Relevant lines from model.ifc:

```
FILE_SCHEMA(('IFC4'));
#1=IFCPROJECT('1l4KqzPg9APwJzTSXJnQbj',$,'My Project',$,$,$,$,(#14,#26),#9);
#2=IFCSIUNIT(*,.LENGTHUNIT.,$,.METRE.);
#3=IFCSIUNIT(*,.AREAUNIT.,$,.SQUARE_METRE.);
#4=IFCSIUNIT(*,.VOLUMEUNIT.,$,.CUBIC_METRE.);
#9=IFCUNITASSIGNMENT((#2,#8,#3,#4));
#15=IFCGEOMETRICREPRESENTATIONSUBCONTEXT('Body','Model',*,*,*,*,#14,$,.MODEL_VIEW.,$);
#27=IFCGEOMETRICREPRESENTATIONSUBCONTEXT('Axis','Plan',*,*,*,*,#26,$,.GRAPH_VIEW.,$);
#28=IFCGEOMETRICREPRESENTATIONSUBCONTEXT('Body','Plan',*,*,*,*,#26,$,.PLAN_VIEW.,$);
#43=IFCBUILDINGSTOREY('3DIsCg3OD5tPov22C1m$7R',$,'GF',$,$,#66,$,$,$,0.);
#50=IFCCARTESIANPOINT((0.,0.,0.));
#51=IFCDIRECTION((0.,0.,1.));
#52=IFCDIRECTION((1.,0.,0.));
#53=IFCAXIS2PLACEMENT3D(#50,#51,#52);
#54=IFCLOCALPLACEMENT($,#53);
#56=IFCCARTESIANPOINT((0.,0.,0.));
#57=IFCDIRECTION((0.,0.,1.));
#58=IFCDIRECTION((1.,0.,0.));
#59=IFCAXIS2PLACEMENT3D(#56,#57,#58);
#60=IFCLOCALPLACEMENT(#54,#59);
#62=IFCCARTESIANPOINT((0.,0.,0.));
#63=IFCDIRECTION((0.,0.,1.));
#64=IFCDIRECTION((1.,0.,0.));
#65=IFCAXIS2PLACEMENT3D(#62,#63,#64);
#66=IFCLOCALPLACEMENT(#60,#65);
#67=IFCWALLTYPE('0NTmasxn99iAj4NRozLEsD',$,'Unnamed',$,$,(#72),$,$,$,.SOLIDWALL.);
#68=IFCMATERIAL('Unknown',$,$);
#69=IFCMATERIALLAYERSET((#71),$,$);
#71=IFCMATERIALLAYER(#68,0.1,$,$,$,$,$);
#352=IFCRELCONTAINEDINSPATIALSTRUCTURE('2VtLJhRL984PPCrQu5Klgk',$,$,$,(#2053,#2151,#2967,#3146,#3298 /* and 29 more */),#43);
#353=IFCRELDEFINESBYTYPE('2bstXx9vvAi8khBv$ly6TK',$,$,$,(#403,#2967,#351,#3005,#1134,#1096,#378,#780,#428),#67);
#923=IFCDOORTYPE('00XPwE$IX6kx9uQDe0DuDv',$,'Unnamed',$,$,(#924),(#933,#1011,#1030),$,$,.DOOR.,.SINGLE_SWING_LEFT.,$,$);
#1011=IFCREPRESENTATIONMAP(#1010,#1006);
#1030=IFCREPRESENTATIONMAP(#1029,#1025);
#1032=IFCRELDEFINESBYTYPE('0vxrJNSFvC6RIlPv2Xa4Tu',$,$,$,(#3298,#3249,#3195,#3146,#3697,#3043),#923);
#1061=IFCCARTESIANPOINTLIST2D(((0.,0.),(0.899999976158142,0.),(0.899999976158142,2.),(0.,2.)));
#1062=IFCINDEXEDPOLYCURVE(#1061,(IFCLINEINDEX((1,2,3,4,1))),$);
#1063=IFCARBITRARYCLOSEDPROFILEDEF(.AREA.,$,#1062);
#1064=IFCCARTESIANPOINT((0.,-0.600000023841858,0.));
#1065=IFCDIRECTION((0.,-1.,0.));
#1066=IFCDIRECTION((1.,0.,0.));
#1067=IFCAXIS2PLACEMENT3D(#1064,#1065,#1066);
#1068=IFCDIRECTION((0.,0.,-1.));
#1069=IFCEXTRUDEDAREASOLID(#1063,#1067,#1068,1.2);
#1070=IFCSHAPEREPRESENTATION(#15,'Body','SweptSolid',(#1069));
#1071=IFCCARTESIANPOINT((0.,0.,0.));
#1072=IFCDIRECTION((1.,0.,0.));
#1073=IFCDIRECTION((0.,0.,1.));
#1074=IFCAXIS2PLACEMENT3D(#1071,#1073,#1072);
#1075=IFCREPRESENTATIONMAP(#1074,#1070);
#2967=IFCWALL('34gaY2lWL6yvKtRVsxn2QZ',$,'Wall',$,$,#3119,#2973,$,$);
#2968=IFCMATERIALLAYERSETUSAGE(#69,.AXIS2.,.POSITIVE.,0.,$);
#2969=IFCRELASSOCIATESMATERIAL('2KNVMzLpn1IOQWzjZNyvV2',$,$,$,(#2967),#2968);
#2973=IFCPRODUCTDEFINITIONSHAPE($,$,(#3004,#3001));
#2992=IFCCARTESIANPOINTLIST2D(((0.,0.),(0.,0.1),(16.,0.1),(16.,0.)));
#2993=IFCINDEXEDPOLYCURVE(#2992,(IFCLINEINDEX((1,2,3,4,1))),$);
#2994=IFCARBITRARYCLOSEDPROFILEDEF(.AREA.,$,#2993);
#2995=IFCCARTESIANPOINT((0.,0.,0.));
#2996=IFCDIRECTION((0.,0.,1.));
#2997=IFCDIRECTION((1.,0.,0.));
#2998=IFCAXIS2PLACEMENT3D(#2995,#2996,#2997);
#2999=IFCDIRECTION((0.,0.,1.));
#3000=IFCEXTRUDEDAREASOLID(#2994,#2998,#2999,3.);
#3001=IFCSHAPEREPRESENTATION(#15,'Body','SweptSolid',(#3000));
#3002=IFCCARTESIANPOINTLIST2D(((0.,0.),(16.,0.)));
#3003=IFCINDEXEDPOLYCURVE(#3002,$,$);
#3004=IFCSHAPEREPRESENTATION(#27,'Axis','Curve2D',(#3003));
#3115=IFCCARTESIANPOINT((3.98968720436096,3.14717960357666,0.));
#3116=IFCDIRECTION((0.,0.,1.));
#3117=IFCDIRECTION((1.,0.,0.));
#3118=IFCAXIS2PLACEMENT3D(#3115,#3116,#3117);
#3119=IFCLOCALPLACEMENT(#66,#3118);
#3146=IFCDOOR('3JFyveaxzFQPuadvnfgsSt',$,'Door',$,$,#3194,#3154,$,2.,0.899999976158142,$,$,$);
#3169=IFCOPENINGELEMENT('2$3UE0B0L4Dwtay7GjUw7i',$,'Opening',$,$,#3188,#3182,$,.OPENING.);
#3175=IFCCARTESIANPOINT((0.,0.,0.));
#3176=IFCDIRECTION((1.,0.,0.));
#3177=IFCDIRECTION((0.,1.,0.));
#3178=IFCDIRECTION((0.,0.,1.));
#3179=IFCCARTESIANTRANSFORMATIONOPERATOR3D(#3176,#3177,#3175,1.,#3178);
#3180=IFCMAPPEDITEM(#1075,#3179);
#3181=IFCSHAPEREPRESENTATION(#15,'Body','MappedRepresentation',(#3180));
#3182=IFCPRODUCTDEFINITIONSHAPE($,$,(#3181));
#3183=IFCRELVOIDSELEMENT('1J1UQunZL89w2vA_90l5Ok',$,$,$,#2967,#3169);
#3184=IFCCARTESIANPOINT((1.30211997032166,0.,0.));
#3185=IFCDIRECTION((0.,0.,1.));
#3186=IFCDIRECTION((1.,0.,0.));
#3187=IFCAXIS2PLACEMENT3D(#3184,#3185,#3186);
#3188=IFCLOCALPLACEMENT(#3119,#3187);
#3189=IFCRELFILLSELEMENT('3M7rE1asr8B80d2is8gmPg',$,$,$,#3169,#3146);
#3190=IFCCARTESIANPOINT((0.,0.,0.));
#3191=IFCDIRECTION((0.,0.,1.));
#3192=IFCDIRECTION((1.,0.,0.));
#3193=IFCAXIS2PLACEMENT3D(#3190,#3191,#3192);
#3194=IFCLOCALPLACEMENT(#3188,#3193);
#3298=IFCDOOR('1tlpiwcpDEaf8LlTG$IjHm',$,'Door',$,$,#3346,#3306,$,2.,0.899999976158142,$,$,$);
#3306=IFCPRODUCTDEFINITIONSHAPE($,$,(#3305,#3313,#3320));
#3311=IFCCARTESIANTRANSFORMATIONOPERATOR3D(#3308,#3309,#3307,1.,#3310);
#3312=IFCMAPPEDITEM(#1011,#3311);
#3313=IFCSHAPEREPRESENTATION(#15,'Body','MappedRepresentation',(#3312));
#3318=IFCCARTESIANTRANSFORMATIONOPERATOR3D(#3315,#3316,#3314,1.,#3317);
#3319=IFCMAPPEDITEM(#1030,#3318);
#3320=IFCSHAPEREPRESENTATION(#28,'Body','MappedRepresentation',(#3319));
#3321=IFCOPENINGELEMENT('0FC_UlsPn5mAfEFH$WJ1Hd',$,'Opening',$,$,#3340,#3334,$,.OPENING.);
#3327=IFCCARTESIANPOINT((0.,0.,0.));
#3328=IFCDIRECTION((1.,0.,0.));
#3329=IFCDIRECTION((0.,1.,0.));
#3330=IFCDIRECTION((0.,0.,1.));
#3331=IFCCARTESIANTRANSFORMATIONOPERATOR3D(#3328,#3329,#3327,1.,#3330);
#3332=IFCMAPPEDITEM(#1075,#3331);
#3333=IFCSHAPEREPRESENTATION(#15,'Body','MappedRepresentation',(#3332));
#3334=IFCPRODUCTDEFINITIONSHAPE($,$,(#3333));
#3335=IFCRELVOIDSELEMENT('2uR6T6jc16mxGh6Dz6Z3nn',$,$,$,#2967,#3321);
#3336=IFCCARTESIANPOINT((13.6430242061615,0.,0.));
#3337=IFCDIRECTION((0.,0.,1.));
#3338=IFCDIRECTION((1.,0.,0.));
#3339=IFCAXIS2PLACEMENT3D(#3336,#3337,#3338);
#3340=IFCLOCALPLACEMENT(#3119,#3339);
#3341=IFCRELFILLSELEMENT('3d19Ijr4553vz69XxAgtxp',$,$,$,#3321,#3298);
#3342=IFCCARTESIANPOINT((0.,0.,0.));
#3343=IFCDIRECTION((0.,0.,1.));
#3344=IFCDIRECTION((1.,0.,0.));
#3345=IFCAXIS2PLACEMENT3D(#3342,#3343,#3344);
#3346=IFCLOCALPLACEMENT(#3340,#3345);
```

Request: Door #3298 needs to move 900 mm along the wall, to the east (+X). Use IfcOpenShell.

```python
import ifcopenshell
import ifcopenshell.api.geometry
import ifcopenshell.util.placement
import ifcopenshell.util.unit

model = ifcopenshell.open("model.ifc")
unit_scale = ifcopenshell.util.unit.calculate_unit_scale(model)

door = model.by_guid("1tlpiwcpDEaf8LlTG$IjHm")
opening = door.FillsVoids[0].RelatingOpeningElement
wall = opening.VoidsElements[0].RelatingBuildingElement

wall_matrix = ifcopenshell.util.placement.get_local_placement(wall.ObjectPlacement)
shift = wall_matrix[:3, 0] * 0.9 / unit_scale
before = ifcopenshell.util.placement.get_local_placement(door.ObjectPlacement)[:3, 3].copy()

# The door is placed relative to its opening, so it follows when the opening moves.
matrix = ifcopenshell.util.placement.get_local_placement(opening.ObjectPlacement)
matrix[:3, 3] += shift
ifcopenshell.api.geometry.edit_object_placement(
    model, product=opening, matrix=matrix, is_si=False, should_transform_children=True
)

after = ifcopenshell.util.placement.get_local_placement(door.ObjectPlacement)[:3, 3]
print("door moved by", (after - before).round(3) + 0.0)

model.write("model_v2.ifc")
```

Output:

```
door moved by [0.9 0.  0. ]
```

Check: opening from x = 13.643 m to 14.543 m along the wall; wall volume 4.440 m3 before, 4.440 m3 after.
